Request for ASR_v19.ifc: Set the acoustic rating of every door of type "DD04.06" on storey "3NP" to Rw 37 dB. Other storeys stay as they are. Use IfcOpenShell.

First a look at what the model holds.

```python
import ifcopenshell
import ifcopenshell.util.element

model = ifcopenshell.open("ASR_v19.ifc")
print(model.schema)
storey = next(s for s in model.by_type("IfcBuildingStorey") if s.Name == "3NP")
doors = [e for e in ifcopenshell.util.element.get_decomposition(storey) if e.is_a("IfcDoor")]
seen = {}
for e in doors:
    element_type = ifcopenshell.util.element.get_type(e)
    key = (element_type.Name if element_type != e and element_type else None, ifcopenshell.util.element.get_pset(e, "Pset_DoorCommon", "AcousticRating"))
    seen[key] = seen.get(key, 0) + 1
for (name, value), count in sorted(seen.items(), key=str):
    print(count, "x", name, "|", value)
```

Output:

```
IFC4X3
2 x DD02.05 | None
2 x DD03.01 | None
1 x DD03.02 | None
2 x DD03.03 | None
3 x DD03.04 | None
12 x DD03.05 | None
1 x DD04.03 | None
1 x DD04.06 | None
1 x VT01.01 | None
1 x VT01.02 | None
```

```python
import ifcopenshell
import ifcopenshell.api.pset
import ifcopenshell.util.element

model = ifcopenshell.open("ASR_v19.ifc")

storey = next(s for s in model.by_type("IfcBuildingStorey") if s.Name == "3NP")
doors = [e for e in ifcopenshell.util.element.get_decomposition(storey) if e.is_a("IfcDoor")]

count = 0
for e in doors:
    element_type = ifcopenshell.util.element.get_type(e)
    if element_type in (None, e) or element_type.Name != "DD04.06":
        continue
    # add_pset returns the element's existing set when there is one.
    pset = ifcopenshell.api.pset.add_pset(model, product=e, name="Pset_DoorCommon")
    ifcopenshell.api.pset.edit_pset(model, pset=pset, properties={"AcousticRating": "Rw 37 dB"})
    count += 1

print(count, "doors updated")

model.write("ASR_v19_v2.ifc")
```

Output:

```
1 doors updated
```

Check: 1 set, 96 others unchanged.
